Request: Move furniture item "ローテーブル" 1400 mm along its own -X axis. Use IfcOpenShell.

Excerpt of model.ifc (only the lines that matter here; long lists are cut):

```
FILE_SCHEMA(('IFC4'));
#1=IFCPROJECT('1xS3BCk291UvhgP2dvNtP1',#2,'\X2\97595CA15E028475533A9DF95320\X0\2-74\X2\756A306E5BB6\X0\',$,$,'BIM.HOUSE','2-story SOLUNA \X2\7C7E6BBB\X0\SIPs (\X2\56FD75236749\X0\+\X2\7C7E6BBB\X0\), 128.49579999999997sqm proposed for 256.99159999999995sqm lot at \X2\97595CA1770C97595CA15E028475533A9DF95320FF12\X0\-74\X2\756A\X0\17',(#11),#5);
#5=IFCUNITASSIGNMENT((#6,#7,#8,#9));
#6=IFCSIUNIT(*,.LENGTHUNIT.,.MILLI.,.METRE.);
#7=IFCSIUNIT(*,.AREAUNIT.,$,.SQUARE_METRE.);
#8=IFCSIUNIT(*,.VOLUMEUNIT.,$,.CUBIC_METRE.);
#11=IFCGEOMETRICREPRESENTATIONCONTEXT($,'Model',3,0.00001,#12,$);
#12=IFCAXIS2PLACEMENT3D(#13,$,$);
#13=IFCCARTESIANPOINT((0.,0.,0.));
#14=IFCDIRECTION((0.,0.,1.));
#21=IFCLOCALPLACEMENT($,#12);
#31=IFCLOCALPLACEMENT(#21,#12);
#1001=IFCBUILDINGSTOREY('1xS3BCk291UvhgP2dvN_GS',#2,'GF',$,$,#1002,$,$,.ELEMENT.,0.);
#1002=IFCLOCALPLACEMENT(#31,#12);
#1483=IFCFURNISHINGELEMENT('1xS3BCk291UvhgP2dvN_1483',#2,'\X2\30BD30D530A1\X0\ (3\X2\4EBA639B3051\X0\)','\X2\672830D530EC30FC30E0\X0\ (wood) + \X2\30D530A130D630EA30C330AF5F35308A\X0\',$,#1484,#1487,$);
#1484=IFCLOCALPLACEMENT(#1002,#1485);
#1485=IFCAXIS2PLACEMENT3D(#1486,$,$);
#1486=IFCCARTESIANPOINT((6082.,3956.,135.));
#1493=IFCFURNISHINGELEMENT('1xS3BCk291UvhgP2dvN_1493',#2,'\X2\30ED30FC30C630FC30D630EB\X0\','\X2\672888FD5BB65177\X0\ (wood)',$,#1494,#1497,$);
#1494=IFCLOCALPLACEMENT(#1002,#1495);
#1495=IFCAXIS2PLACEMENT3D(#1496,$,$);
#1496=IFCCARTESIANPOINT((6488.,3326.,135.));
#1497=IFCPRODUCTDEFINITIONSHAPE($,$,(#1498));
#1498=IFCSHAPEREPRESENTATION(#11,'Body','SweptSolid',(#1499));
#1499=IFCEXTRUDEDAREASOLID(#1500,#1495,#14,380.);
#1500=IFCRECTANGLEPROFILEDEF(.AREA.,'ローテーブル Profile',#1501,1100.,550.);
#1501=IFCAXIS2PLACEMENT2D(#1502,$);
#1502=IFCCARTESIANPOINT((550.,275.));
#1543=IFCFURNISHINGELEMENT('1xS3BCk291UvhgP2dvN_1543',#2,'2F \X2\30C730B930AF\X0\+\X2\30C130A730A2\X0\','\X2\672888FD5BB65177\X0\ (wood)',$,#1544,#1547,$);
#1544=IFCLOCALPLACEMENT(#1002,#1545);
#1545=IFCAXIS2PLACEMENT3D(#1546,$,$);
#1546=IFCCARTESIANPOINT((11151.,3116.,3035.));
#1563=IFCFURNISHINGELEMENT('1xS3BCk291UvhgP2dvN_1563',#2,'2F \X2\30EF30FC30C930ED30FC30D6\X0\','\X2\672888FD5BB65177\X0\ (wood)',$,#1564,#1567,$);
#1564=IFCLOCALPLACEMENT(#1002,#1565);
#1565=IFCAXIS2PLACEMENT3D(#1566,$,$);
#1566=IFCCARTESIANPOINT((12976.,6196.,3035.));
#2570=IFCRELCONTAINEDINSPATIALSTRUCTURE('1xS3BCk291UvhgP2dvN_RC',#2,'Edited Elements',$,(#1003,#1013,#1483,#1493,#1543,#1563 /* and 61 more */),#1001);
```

```python
import ifcopenshell
import ifcopenshell.api.geometry
import ifcopenshell.util.placement
import ifcopenshell.util.unit

model = ifcopenshell.open("model.ifc")
unit_scale = ifcopenshell.util.unit.calculate_unit_scale(model)

item = model.by_guid("1xS3BCk291UvhgP2dvN_1493")
matrix = ifcopenshell.util.placement.get_local_placement(item.ObjectPlacement)
matrix[:3, 3] -= matrix[:3, 0] * 1.4 / unit_scale
ifcopenshell.api.geometry.edit_object_placement(model, product=item, matrix=matrix, is_si=False)

print(ifcopenshell.util.placement.get_local_placement(item.ObjectPlacement).round(3) + 0.0)

model.write("model_edited.ifc")
```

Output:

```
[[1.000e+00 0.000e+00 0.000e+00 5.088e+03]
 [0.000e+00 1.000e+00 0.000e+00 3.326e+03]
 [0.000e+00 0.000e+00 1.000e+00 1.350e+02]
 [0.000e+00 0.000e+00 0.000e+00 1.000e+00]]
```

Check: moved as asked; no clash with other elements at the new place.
